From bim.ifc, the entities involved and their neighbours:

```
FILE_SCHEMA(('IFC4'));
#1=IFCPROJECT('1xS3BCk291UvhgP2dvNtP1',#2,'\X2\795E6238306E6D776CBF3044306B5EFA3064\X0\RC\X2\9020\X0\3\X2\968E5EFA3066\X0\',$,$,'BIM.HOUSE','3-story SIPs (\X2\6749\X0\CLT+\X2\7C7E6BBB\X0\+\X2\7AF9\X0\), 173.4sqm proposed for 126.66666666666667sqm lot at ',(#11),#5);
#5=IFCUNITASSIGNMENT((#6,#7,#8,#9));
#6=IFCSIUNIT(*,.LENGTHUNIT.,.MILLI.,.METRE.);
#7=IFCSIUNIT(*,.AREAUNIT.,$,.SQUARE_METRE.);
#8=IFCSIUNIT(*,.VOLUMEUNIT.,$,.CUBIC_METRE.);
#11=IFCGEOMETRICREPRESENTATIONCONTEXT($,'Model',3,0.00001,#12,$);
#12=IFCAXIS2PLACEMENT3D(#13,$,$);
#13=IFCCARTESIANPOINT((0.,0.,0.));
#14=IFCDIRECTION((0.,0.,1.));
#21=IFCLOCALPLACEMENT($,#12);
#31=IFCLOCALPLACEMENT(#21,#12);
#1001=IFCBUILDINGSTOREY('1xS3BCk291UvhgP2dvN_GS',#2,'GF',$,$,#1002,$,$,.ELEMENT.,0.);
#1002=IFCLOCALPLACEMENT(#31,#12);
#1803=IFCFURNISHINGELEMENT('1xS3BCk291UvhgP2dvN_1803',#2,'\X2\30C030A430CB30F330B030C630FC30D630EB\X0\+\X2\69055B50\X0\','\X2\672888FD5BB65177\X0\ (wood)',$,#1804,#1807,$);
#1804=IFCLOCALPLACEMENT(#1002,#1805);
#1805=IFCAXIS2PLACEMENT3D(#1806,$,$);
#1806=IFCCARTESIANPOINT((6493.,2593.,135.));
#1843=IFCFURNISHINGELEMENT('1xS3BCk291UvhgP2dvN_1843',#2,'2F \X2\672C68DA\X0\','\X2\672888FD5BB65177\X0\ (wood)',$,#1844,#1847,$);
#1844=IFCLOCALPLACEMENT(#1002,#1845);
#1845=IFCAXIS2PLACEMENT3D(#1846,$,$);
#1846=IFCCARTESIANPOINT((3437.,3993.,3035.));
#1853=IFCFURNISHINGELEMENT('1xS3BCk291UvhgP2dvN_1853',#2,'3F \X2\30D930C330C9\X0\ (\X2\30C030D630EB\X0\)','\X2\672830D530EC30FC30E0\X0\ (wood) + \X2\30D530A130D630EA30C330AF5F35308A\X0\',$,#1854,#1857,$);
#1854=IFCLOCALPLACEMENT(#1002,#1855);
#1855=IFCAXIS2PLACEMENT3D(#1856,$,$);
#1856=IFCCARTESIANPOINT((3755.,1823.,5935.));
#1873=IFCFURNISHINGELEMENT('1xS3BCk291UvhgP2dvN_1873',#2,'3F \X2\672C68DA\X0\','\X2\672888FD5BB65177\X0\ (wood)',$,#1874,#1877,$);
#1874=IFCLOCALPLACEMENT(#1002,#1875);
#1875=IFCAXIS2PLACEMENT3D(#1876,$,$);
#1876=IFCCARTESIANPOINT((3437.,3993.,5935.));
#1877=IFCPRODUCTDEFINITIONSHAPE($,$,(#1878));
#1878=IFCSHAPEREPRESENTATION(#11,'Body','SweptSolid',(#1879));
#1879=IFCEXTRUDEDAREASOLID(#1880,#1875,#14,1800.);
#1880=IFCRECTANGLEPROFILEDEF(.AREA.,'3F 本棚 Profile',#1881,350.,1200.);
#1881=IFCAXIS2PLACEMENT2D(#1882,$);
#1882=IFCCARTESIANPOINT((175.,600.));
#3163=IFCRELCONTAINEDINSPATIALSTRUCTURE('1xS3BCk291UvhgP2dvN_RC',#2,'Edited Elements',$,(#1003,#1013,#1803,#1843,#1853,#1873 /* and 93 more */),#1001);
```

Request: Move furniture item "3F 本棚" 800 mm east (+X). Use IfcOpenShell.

```python
import ifcopenshell
import ifcopenshell.api.geometry
import ifcopenshell.util.placement

model = ifcopenshell.open("bim.ifc")

item = model.by_guid("1xS3BCk291UvhgP2dvN_1873")
matrix = ifcopenshell.util.placement.get_local_placement(item.ObjectPlacement)
matrix[0, 3] += 800.0
ifcopenshell.api.geometry.edit_object_placement(model, product=item, matrix=matrix, is_si=False)

print(ifcopenshell.util.placement.get_local_placement(item.ObjectPlacement).round(3) + 0.0)

model.write("bim_updated.ifc")
```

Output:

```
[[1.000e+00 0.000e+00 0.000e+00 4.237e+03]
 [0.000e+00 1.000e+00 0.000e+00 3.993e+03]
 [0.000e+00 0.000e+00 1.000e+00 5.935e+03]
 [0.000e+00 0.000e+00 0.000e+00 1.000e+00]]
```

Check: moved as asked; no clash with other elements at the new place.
